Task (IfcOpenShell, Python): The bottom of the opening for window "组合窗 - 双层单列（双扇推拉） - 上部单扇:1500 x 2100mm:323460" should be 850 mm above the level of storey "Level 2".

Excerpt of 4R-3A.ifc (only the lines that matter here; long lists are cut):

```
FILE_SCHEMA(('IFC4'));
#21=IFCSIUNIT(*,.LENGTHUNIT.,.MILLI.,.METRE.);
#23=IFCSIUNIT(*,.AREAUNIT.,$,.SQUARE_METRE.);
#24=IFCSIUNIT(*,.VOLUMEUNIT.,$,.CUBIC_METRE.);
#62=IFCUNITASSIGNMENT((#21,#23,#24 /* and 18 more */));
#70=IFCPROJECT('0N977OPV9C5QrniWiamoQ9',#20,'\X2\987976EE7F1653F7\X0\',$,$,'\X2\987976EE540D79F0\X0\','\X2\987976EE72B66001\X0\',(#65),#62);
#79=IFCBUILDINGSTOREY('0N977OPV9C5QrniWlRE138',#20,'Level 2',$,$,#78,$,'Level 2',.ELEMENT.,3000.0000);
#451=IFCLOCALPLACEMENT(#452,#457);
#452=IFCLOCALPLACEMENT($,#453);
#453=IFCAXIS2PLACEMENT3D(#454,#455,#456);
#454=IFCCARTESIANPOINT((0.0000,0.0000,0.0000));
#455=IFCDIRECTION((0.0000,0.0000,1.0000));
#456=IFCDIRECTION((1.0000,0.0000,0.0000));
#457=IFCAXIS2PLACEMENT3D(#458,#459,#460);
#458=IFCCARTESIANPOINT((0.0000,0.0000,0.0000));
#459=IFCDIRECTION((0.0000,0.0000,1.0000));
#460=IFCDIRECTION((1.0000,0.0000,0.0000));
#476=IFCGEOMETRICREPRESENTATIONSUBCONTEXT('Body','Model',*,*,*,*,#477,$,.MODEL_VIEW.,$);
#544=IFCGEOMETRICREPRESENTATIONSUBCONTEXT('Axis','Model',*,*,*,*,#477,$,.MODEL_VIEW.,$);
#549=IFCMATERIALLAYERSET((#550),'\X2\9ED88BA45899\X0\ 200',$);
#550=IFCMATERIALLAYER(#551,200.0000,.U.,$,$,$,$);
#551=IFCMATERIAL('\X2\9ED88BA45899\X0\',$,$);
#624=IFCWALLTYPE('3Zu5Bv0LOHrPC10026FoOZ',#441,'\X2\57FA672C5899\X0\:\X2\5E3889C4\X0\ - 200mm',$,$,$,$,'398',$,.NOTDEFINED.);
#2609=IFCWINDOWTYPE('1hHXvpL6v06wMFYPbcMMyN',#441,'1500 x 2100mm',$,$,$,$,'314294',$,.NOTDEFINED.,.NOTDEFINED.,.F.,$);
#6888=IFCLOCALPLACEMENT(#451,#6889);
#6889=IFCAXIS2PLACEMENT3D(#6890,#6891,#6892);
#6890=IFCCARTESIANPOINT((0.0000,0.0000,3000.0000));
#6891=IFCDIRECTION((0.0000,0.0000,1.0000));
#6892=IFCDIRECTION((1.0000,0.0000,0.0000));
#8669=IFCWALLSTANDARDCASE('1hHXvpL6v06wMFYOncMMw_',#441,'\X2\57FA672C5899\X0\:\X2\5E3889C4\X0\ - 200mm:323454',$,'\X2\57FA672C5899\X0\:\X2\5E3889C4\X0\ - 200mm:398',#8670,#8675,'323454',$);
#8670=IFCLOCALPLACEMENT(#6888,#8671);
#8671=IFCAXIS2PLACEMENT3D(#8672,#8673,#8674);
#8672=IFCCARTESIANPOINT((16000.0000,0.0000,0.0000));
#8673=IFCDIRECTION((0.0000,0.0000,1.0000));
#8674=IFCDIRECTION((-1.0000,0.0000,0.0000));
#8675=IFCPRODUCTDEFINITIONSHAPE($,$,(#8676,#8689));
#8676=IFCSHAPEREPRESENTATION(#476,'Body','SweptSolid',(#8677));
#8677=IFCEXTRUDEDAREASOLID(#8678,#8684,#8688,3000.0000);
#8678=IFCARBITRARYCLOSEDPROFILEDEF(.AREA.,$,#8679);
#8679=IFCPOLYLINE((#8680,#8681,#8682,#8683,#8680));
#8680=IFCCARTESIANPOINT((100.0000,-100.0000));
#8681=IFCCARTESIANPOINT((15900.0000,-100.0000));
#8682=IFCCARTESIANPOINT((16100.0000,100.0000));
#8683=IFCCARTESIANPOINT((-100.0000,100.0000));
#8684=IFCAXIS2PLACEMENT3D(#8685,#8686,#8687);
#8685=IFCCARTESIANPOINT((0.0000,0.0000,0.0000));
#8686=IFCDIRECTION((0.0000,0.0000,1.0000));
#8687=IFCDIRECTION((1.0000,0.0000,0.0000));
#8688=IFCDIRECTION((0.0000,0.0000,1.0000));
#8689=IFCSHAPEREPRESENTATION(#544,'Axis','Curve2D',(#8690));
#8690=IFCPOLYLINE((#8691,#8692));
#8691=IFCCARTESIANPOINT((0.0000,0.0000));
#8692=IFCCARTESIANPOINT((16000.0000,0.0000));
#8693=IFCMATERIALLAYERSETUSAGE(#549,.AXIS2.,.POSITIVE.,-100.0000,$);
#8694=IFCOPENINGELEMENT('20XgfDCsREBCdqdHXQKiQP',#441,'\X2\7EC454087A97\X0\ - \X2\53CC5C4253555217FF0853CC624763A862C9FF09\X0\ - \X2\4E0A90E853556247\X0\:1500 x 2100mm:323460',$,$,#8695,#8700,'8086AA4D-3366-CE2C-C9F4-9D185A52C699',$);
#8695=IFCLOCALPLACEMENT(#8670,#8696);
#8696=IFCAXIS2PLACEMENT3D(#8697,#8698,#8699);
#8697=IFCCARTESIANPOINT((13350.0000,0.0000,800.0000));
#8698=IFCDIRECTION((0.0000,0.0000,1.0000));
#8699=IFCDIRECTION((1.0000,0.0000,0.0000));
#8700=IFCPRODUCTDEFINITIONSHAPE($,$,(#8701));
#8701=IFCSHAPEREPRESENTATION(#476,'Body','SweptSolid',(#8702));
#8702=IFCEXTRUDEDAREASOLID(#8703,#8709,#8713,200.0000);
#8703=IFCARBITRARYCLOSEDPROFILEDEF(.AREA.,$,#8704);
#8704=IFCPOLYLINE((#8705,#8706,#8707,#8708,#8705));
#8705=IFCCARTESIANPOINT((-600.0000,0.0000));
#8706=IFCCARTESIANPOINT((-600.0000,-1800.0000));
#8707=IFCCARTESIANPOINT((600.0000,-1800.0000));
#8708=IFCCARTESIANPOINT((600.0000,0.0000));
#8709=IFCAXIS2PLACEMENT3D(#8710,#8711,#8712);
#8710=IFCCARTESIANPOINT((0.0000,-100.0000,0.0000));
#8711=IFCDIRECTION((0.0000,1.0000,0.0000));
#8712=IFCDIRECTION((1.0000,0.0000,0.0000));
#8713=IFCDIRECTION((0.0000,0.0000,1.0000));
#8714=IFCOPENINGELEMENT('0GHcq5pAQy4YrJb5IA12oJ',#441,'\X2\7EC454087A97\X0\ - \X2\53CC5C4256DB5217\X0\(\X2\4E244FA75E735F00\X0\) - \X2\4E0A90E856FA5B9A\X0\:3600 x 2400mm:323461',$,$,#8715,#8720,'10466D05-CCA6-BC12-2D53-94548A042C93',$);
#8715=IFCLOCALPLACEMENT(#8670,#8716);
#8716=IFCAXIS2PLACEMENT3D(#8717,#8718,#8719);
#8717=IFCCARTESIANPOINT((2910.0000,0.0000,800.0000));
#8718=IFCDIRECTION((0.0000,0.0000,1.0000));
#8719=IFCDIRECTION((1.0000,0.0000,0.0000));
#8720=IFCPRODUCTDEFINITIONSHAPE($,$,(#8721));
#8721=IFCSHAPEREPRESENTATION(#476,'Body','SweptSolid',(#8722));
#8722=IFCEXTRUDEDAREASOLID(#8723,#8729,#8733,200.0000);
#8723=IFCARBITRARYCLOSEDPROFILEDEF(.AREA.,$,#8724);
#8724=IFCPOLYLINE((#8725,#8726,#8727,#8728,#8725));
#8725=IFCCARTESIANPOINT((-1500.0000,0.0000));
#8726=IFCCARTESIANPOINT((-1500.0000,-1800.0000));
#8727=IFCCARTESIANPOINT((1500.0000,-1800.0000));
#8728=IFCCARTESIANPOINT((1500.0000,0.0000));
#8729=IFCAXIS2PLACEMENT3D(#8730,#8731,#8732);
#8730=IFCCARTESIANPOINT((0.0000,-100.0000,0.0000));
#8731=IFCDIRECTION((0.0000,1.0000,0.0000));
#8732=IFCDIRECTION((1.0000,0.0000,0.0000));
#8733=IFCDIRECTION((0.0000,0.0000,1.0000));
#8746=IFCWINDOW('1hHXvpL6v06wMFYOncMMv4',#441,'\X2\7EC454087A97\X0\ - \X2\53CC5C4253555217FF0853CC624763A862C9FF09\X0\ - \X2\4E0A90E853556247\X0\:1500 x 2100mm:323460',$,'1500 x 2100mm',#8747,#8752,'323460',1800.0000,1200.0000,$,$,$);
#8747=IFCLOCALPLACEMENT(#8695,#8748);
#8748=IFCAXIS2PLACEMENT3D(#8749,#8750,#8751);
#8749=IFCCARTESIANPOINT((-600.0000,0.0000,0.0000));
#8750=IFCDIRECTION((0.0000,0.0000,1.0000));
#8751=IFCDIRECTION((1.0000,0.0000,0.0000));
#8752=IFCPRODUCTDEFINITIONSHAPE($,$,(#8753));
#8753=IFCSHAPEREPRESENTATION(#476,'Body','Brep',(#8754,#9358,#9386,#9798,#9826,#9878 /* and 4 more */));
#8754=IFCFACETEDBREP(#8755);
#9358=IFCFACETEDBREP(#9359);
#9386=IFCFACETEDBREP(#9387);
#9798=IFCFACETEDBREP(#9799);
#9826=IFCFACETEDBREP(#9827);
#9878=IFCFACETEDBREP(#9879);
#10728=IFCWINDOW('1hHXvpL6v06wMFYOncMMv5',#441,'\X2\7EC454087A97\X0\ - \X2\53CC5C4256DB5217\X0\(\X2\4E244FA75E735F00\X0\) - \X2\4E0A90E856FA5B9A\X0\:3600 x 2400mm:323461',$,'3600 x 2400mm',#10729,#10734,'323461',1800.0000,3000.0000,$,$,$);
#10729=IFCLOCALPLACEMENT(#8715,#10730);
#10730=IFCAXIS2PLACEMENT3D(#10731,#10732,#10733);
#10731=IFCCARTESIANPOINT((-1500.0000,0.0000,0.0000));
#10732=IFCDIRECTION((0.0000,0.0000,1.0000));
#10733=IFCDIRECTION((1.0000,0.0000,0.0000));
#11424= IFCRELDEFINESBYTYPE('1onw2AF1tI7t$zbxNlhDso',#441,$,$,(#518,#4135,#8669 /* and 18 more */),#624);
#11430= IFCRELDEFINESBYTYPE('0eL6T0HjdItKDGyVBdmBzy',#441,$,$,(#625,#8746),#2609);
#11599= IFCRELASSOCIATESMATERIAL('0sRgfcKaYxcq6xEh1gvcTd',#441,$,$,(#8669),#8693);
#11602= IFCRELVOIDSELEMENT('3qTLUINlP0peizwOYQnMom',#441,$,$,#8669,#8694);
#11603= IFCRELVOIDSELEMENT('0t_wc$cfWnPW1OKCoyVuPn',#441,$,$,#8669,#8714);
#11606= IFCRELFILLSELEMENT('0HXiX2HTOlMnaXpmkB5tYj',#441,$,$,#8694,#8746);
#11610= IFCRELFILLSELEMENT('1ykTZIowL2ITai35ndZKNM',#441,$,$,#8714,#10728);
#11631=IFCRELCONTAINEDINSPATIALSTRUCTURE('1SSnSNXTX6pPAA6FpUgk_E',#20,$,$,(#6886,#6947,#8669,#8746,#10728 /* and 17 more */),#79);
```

```python
import numpy as np
import ifcopenshell
import ifcopenshell.api.geometry
import ifcopenshell.geom
import ifcopenshell.util.element
import ifcopenshell.util.placement
import ifcopenshell.util.shape
import ifcopenshell.util.unit

model = ifcopenshell.open("4R-3A.ifc")
unit_scale = ifcopenshell.util.unit.calculate_unit_scale(model)

window = model.by_guid("1hHXvpL6v06wMFYOncMMv4")
opening = window.FillsVoids[0].RelatingOpeningElement
storey = ifcopenshell.util.element.get_container(window, ifc_class="IfcBuildingStorey")
level = ifcopenshell.util.placement.get_local_placement(storey.ObjectPlacement)[2, 3]

# The opening's origin need not be at the sill, so measure its lowest point.
shape = ifcopenshell.geom.create_shape(ifcopenshell.geom.settings(), opening)
bottom = ifcopenshell.util.shape.get_shape_bottom_elevation(shape, shape.geometry) / unit_scale
dz = level + 0.85 / unit_scale - bottom

shift = np.array([0.0, 0.0, dz])
# The window is placed relative to its opening, so it follows when the opening moves.
matrix = ifcopenshell.util.placement.get_local_placement(opening.ObjectPlacement)
matrix[:3, 3] += shift
ifcopenshell.api.geometry.edit_object_placement(
    model, product=opening, matrix=matrix, is_si=False, should_transform_children=True
)

print(f"moved by {dz * unit_scale:+.3f} m")

model.write("4R-3A_rev.ifc")
```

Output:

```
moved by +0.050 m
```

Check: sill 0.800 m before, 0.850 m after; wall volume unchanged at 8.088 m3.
